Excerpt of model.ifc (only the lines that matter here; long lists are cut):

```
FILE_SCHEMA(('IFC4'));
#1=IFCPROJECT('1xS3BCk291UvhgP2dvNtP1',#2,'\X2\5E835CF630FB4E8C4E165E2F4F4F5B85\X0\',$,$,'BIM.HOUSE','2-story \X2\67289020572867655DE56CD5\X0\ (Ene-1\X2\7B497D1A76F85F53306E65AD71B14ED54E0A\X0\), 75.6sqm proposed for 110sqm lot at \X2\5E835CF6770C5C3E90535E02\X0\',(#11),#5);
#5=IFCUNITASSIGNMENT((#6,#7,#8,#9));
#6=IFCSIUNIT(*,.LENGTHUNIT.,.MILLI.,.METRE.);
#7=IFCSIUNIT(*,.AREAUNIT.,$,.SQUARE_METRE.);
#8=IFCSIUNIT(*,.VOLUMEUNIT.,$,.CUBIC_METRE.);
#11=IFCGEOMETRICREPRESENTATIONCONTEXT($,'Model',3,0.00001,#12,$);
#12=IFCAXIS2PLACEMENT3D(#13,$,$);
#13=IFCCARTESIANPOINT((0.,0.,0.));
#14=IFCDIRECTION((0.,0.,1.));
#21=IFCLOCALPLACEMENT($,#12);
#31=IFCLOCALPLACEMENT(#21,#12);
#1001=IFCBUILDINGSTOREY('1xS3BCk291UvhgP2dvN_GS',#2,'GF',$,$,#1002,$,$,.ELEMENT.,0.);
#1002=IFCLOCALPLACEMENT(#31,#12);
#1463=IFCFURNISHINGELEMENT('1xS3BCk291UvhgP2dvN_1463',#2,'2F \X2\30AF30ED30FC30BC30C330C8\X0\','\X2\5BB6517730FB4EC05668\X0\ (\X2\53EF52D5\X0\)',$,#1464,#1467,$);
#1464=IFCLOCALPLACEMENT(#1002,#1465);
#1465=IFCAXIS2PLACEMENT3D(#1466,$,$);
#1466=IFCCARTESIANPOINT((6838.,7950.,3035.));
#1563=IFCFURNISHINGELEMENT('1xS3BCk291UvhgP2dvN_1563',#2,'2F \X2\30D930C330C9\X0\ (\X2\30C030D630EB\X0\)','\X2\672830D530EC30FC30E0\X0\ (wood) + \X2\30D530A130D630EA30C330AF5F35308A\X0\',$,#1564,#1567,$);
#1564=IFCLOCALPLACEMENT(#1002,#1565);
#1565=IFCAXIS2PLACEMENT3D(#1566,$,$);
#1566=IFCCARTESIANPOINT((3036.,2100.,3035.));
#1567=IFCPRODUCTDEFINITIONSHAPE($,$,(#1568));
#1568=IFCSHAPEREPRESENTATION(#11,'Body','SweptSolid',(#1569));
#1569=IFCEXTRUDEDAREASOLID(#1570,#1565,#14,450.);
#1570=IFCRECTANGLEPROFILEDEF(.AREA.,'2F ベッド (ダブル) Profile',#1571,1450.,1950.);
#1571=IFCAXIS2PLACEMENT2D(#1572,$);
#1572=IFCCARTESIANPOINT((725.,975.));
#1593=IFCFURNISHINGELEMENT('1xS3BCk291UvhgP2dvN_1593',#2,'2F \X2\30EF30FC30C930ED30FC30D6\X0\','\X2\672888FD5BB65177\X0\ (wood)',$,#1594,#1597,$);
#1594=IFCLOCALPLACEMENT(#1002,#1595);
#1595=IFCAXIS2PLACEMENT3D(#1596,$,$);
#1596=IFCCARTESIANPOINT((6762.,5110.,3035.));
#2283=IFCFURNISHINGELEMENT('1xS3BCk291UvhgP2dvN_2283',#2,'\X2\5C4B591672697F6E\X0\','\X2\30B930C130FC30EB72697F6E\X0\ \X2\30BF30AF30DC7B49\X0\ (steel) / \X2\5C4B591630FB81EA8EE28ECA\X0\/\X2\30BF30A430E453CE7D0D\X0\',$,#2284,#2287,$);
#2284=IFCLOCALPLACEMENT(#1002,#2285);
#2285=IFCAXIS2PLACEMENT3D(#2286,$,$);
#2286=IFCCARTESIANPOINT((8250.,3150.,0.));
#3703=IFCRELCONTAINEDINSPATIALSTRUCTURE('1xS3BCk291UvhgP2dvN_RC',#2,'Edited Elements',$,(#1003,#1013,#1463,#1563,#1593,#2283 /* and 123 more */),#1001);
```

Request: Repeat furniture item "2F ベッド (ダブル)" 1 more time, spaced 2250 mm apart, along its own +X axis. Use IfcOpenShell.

```python
import ifcopenshell
import ifcopenshell.api.geometry
import ifcopenshell.api.root
import ifcopenshell.util.element
import ifcopenshell.util.placement

model = ifcopenshell.open("model.ifc")


def reuse_history(source, copy):
    """copy_class also copies each property set's owner history, people and application; keep the originals."""
    for rel in copy.IsDefinedBy:
        if rel.is_a("IfcRelDefinesByProperties") and (history := rel.RelatingPropertyDefinition.OwnerHistory):
            rel.RelatingPropertyDefinition.OwnerHistory = source.OwnerHistory
            ifcopenshell.util.element.remove_deep2(model, history)


source = model.by_guid("1xS3BCk291UvhgP2dvN_1563")
base = ifcopenshell.util.placement.get_local_placement(source.ObjectPlacement)
step = base[:3, 0] * 2250.0

for i in range(1, 2):
    copy = ifcopenshell.api.root.copy_class(model, product=source)
    copy.Representation = ifcopenshell.util.element.copy_deep(
        model, source.Representation, exclude=["IfcGeometricRepresentationContext", "IfcRepresentationMap"]
    )
    reuse_history(source, copy)
    matrix = base.copy()
    matrix[:3, 3] += i * step
    print("added at", matrix[:3, 3].round(3) + 0.0)
    ifcopenshell.api.geometry.edit_object_placement(model, product=copy, matrix=matrix, is_si=False)

model.write("model_updated.ifc")
```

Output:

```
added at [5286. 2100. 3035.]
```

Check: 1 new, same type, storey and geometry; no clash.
